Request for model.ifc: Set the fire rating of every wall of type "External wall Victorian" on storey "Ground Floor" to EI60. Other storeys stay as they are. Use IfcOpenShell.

First a look at what the model holds.

```python
import ifcopenshell
import ifcopenshell.util.element

model = ifcopenshell.open("model.ifc")
print(model.schema)
storey = next(s for s in model.by_type("IfcBuildingStorey") if s.Name == "Ground Floor")
walls = [e for e in ifcopenshell.util.element.get_decomposition(storey) if e.is_a("IfcWall")]
seen = {}
for e in walls:
    element_type = ifcopenshell.util.element.get_type(e)
    key = (element_type.Name if element_type != e and element_type else None, ifcopenshell.util.element.get_pset(e, "Pset_WallCommon", "FireRating"))
    seen[key] = seen.get(key, 0) + 1
for (name, value), count in sorted(seen.items(), key=str):
    print(count, "x", name, "|", value)
```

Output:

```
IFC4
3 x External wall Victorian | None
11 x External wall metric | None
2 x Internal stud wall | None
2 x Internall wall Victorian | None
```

```python
import ifcopenshell
import ifcopenshell.api.pset
import ifcopenshell.util.element

model = ifcopenshell.open("model.ifc")

storey = next(s for s in model.by_type("IfcBuildingStorey") if s.Name == "Ground Floor")
walls = [e for e in ifcopenshell.util.element.get_decomposition(storey) if e.is_a("IfcWall")]

count = 0
for e in walls:
    element_type = ifcopenshell.util.element.get_type(e)
    if element_type in (None, e) or element_type.Name != "External wall Victorian":
        continue
    # add_pset returns the element's existing set when there is one.
    pset = ifcopenshell.api.pset.add_pset(model, product=e, name="Pset_WallCommon")
    ifcopenshell.api.pset.edit_pset(model, pset=pset, properties={"FireRating": "EI60"})
    count += 1

print(count, "walls updated")

model.write("model_v2.ifc")
```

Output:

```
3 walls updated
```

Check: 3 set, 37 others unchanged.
